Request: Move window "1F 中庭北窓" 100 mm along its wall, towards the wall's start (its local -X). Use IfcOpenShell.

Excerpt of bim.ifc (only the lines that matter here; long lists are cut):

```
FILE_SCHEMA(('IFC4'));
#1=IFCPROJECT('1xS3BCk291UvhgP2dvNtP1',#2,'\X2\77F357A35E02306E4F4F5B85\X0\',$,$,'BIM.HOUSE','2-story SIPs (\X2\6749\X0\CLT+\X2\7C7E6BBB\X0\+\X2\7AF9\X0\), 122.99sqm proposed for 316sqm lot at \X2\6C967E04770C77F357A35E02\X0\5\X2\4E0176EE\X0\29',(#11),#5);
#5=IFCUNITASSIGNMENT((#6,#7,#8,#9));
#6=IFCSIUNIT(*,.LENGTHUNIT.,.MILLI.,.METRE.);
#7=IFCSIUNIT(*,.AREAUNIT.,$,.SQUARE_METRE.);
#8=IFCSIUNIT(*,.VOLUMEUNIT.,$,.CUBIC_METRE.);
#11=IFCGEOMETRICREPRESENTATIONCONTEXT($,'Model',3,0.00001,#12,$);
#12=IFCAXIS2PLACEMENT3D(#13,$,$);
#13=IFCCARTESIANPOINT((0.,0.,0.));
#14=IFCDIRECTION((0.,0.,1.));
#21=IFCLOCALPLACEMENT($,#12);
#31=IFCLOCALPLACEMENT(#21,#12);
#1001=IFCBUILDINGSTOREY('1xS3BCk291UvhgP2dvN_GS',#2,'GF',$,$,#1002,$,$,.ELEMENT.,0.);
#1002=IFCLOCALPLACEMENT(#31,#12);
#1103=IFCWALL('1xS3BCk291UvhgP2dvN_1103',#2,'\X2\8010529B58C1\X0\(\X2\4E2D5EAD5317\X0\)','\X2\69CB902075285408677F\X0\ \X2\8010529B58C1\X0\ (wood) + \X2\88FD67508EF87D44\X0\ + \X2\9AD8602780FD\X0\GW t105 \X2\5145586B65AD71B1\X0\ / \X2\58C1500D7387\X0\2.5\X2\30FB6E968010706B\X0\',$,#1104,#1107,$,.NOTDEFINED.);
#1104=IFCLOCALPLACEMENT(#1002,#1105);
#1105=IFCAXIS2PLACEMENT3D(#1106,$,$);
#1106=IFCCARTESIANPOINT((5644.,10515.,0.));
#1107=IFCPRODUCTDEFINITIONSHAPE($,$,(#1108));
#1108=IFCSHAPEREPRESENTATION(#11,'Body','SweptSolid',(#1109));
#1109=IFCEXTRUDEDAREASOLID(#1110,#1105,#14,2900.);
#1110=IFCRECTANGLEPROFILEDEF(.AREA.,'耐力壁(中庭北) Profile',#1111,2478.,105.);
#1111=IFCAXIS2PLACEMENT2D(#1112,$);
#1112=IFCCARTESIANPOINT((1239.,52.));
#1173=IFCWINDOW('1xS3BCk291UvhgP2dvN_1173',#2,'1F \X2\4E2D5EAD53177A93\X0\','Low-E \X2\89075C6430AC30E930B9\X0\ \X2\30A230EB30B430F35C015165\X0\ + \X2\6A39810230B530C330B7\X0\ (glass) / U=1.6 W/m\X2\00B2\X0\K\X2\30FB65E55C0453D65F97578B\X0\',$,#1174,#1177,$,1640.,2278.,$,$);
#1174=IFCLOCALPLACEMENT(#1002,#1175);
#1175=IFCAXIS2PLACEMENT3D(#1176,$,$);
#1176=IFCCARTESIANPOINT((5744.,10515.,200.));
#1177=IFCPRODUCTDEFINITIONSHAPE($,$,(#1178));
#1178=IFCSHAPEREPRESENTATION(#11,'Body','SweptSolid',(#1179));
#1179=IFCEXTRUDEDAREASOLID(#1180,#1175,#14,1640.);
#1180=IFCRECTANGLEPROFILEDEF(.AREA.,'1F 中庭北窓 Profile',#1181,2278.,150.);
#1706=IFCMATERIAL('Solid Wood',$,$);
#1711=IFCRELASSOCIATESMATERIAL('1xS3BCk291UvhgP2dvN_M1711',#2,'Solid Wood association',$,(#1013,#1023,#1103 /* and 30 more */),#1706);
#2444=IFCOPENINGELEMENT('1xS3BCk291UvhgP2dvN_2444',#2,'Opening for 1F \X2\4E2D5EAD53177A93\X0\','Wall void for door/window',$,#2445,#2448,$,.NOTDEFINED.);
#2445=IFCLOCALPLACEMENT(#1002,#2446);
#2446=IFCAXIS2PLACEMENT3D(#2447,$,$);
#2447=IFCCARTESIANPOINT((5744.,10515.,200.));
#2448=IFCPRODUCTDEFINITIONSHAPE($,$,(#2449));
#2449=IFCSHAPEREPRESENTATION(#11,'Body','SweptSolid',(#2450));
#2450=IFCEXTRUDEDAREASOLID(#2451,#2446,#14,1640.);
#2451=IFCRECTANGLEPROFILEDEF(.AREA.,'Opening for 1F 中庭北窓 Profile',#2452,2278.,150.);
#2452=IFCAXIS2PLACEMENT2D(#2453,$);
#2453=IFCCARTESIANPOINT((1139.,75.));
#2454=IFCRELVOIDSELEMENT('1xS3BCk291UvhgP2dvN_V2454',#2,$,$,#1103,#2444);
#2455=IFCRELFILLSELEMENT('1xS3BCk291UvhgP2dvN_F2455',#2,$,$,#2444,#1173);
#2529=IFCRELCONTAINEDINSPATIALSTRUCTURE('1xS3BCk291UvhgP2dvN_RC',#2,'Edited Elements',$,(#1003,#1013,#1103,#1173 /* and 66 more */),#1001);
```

```python
import ifcopenshell
import ifcopenshell.api.geometry
import ifcopenshell.util.placement

model = ifcopenshell.open("bim.ifc")

window = model.by_guid("1xS3BCk291UvhgP2dvN_1173")
opening = window.FillsVoids[0].RelatingOpeningElement
wall = opening.VoidsElements[0].RelatingBuildingElement

wall_matrix = ifcopenshell.util.placement.get_local_placement(wall.ObjectPlacement)
shift = wall_matrix[:3, 0] * -100.0
before = ifcopenshell.util.placement.get_local_placement(window.ObjectPlacement)[:3, 3].copy()

# The window is not placed relative to its opening, so move both.
for product in (opening, window):
    matrix = ifcopenshell.util.placement.get_local_placement(product.ObjectPlacement)
    matrix[:3, 3] += shift
    ifcopenshell.api.geometry.edit_object_placement(model, product=product, matrix=matrix, is_si=False)

after = ifcopenshell.util.placement.get_local_placement(window.ObjectPlacement)[:3, 3]
print("window moved by", (after - before).round(3) + 0.0)

model.write("bim_edited.ifc")
```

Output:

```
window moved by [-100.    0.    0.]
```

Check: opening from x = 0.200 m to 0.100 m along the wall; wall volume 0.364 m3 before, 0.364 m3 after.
